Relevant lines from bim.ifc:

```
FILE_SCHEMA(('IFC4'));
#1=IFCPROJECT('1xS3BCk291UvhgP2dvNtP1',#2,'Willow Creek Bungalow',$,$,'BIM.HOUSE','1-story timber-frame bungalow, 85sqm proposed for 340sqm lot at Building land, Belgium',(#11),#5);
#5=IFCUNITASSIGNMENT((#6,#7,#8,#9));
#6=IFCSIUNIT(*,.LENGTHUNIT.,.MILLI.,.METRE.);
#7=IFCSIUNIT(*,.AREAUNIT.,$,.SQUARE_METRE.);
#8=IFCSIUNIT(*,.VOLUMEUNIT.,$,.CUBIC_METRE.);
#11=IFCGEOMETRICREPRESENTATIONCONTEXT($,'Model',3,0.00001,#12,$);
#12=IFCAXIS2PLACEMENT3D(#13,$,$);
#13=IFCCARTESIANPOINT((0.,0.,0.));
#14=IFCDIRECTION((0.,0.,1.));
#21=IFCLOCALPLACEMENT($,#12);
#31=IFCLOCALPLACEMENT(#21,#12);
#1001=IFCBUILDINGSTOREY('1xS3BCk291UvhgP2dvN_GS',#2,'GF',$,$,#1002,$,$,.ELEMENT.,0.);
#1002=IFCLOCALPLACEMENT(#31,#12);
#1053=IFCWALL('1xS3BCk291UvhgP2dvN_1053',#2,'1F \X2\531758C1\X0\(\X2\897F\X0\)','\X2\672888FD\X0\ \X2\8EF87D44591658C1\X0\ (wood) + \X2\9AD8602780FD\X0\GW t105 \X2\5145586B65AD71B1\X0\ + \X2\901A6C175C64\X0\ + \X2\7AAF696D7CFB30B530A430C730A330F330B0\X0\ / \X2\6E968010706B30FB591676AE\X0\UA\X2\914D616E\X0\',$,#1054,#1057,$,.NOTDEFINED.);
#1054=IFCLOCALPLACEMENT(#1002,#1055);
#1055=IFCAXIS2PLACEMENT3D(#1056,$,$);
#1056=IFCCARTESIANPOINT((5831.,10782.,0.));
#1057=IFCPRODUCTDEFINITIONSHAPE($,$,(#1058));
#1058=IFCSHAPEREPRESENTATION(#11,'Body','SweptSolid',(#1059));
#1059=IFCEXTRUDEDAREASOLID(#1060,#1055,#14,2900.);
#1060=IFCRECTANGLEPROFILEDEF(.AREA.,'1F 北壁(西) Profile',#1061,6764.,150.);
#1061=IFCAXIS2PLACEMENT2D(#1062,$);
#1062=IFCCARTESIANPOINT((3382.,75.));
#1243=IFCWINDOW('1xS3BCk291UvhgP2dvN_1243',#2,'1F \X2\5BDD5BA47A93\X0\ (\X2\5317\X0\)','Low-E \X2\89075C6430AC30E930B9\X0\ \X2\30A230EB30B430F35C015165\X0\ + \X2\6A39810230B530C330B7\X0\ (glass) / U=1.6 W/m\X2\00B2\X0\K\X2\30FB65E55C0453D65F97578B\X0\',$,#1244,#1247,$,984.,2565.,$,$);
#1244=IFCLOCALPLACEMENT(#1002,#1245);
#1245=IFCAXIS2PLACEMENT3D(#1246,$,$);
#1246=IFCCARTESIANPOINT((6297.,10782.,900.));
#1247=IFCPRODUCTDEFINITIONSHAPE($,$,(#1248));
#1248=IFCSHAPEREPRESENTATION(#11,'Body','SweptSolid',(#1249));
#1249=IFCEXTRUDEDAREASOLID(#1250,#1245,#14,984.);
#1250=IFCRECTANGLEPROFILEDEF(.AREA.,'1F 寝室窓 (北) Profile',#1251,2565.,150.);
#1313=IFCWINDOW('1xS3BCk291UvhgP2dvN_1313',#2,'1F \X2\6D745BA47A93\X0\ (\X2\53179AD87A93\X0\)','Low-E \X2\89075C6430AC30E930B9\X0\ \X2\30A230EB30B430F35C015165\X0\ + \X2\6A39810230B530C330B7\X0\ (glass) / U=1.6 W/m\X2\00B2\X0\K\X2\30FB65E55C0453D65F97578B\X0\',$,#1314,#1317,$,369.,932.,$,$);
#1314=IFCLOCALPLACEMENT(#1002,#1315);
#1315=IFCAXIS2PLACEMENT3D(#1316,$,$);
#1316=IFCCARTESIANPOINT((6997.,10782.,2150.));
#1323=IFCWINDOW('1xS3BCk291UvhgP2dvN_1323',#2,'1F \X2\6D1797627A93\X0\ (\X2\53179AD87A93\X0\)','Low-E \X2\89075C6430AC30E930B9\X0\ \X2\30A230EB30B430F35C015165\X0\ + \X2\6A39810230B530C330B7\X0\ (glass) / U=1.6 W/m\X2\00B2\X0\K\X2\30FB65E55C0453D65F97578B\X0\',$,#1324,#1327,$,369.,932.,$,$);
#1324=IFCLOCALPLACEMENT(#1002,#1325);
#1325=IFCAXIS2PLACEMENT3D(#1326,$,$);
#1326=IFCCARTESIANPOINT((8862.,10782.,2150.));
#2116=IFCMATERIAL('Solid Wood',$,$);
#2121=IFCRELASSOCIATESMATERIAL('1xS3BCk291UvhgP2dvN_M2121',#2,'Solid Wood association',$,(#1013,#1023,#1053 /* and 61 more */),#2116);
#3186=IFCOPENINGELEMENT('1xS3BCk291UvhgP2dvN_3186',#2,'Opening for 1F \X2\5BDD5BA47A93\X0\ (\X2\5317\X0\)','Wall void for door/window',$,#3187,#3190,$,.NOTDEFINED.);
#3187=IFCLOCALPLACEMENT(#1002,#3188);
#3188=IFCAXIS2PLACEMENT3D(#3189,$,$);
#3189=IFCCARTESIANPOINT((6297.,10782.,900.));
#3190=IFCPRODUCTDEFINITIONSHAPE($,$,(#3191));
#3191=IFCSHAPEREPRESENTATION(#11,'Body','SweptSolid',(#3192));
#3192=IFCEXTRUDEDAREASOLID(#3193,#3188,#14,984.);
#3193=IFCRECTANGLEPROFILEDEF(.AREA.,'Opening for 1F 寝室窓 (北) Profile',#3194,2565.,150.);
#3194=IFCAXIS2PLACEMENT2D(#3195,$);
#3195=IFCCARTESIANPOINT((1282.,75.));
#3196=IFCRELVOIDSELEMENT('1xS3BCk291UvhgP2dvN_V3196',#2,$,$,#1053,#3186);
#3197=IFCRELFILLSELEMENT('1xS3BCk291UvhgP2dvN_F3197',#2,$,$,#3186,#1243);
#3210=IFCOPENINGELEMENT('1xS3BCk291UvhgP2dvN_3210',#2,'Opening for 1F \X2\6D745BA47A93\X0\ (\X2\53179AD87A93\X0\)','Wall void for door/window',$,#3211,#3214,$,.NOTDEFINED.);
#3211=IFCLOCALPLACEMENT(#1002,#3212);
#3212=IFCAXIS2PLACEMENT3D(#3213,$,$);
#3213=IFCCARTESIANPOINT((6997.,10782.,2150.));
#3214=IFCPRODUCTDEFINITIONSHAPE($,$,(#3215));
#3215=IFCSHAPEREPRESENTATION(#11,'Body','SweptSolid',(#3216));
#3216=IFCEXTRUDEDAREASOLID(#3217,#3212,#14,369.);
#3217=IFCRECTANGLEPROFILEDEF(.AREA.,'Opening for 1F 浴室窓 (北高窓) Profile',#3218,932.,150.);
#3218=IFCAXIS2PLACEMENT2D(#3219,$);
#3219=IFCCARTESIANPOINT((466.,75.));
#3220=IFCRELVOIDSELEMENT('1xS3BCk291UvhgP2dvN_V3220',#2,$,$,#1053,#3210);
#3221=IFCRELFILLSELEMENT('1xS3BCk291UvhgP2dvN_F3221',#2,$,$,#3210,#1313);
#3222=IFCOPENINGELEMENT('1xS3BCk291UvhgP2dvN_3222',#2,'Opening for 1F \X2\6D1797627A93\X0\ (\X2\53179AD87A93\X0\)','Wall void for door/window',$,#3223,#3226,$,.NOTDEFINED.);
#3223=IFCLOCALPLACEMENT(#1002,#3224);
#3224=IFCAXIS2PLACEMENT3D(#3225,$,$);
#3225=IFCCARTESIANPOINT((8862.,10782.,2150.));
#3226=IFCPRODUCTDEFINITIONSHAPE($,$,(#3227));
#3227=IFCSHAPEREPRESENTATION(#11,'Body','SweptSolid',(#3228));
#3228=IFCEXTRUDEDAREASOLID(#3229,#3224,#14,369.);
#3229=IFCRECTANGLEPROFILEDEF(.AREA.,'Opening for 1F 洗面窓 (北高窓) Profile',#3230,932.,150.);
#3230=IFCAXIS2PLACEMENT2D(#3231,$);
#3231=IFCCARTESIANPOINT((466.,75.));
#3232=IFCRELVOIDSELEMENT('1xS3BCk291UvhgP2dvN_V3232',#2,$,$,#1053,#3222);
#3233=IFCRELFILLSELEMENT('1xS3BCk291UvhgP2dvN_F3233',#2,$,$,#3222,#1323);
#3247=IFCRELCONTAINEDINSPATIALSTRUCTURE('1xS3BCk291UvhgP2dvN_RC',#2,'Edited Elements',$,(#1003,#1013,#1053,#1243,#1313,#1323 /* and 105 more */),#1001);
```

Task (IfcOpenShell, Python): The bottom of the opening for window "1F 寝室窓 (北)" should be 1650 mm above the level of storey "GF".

```python
import numpy as np
import ifcopenshell
import ifcopenshell.api.geometry
import ifcopenshell.geom
import ifcopenshell.util.element
import ifcopenshell.util.placement
import ifcopenshell.util.shape
import ifcopenshell.util.unit

model = ifcopenshell.open("bim.ifc")
unit_scale = ifcopenshell.util.unit.calculate_unit_scale(model)

window = model.by_id(1243)
opening = window.FillsVoids[0].RelatingOpeningElement
storey = ifcopenshell.util.element.get_container(window, ifc_class="IfcBuildingStorey")
level = ifcopenshell.util.placement.get_local_placement(storey.ObjectPlacement)[2, 3]

# The opening's origin need not be at the sill, so measure its lowest point.
shape = ifcopenshell.geom.create_shape(ifcopenshell.geom.settings(), opening)
bottom = ifcopenshell.util.shape.get_shape_bottom_elevation(shape, shape.geometry) / unit_scale
dz = level + 1.65 / unit_scale - bottom

shift = np.array([0.0, 0.0, dz])
# The window is not placed relative to its opening, so move both.
for product in (opening, window):
    matrix = ifcopenshell.util.placement.get_local_placement(product.ObjectPlacement)
    matrix[:3, 3] += shift
    ifcopenshell.api.geometry.edit_object_placement(model, product=product, matrix=matrix, is_si=False)

print(f"moved by {dz * unit_scale:+.3f} m")

model.write("bim_edited.ifc")
```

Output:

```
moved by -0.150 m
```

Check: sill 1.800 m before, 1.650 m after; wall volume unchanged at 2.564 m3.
